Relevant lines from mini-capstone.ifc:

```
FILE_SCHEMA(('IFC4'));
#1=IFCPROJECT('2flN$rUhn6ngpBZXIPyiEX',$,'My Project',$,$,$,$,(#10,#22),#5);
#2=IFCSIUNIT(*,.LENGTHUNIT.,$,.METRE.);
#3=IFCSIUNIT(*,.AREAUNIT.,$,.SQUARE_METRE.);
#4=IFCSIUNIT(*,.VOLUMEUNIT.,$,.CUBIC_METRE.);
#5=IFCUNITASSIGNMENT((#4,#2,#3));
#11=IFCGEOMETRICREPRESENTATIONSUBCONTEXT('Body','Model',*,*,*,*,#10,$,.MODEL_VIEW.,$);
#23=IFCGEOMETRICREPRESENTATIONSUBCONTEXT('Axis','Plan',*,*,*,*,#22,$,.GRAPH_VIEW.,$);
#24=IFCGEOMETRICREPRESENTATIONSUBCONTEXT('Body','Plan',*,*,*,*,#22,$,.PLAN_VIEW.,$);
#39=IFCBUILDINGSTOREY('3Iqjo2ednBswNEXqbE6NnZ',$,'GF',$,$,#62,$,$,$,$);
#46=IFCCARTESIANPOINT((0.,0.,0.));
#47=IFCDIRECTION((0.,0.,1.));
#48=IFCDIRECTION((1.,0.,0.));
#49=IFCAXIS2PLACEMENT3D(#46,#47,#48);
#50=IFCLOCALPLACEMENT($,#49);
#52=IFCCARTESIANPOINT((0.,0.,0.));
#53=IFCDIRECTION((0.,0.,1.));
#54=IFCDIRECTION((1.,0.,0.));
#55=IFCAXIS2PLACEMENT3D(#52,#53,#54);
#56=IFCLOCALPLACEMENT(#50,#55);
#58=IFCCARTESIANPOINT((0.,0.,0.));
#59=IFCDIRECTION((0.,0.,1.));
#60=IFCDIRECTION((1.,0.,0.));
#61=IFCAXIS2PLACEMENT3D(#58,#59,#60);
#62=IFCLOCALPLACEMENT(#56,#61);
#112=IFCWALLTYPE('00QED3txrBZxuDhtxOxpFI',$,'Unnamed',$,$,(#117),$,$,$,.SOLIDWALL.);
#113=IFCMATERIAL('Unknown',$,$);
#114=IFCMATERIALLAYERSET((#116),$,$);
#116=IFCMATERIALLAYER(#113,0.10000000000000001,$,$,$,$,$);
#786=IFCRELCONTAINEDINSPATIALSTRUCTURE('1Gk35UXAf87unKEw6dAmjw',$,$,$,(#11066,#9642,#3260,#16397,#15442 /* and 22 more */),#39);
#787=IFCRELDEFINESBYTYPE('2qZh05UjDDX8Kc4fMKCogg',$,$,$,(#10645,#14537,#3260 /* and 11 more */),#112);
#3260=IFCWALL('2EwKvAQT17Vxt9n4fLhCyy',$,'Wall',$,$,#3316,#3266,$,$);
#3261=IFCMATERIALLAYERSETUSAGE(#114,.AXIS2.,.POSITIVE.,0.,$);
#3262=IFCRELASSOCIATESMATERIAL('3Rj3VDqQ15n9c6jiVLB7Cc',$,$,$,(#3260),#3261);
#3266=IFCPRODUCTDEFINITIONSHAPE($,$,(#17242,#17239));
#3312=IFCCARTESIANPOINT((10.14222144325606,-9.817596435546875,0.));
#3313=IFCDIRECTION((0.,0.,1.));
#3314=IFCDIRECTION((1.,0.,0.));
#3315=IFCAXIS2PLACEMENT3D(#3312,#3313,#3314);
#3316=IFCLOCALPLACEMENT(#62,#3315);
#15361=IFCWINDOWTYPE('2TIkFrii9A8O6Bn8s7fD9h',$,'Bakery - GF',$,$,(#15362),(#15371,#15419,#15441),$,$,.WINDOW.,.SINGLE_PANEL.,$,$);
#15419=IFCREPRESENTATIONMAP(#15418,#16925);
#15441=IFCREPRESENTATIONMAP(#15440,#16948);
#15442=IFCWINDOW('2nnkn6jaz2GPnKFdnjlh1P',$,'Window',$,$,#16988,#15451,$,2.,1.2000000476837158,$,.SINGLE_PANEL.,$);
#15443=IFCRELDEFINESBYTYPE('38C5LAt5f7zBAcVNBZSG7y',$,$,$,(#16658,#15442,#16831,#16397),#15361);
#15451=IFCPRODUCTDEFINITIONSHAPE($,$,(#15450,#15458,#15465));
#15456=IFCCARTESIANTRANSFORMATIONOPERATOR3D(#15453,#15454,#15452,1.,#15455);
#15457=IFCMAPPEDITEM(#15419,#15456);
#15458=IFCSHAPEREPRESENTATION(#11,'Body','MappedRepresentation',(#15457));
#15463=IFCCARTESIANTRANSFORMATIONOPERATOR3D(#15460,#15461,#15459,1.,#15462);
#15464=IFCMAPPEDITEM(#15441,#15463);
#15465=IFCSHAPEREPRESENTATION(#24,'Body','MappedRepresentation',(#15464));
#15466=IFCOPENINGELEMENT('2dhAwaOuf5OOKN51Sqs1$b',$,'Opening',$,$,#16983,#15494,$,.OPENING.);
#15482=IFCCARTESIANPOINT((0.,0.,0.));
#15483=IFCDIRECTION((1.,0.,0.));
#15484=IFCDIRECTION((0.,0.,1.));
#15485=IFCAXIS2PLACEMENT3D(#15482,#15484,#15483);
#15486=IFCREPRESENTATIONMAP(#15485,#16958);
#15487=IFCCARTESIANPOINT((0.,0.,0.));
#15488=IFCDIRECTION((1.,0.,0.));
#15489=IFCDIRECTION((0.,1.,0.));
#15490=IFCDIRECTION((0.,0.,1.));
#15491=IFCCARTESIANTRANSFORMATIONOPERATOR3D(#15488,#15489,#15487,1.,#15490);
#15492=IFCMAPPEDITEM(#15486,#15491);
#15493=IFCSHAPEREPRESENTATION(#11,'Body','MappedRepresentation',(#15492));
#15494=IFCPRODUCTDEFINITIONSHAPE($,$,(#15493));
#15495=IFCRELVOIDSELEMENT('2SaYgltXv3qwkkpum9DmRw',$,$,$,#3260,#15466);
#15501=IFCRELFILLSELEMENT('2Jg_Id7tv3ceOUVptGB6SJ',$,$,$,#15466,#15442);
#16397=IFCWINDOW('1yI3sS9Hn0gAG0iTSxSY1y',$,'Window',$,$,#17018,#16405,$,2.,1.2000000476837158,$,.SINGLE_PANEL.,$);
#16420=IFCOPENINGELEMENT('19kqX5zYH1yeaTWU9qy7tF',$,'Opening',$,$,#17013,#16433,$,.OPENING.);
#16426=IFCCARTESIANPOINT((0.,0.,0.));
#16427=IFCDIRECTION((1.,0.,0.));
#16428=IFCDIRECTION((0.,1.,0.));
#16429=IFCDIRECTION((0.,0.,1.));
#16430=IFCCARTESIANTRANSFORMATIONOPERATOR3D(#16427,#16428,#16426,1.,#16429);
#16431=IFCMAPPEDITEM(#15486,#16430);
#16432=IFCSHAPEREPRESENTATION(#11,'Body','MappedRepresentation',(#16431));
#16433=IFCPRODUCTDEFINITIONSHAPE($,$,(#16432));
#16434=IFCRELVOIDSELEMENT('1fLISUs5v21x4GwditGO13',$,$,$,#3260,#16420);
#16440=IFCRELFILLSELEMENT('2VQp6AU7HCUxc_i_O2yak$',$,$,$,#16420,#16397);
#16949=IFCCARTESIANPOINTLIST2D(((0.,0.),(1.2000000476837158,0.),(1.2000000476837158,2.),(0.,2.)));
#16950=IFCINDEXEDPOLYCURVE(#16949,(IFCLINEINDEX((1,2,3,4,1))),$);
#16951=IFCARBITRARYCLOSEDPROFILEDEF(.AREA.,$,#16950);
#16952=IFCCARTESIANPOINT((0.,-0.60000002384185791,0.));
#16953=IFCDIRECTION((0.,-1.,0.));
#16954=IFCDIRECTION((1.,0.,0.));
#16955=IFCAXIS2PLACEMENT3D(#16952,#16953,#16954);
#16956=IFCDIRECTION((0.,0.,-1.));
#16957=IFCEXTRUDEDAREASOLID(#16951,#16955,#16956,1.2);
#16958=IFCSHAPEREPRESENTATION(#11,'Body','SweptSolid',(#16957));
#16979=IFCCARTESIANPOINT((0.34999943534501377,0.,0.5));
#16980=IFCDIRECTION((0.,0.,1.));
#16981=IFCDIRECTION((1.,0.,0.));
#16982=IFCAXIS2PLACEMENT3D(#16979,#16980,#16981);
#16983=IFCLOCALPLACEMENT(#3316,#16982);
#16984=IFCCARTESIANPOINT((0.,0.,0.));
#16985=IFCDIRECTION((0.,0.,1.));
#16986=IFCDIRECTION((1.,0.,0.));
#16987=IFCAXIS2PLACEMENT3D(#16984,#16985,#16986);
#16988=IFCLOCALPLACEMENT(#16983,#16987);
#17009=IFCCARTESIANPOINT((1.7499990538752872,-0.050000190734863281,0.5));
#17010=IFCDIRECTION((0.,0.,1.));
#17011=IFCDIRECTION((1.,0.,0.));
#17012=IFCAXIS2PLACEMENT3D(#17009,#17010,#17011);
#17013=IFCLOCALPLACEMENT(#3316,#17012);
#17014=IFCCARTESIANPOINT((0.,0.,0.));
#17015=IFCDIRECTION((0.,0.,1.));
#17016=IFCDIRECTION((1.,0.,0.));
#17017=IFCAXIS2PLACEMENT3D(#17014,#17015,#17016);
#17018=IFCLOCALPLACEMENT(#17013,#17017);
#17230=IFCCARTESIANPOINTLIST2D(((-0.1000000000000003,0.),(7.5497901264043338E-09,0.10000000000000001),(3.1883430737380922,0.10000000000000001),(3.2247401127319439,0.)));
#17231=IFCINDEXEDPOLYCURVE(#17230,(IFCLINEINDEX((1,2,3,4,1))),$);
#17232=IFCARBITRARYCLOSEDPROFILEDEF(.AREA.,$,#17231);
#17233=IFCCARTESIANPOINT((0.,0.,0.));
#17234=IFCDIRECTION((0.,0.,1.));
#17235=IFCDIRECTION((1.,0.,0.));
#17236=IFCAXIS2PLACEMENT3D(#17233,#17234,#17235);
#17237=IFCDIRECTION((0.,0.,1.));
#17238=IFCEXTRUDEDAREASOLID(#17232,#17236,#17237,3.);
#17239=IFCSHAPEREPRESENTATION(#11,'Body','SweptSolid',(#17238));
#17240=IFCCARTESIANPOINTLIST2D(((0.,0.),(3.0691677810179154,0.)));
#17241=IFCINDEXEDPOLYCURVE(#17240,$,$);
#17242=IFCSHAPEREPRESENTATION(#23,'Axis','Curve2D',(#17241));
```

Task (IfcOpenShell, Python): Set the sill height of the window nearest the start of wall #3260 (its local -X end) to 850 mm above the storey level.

```python
import numpy as np
import ifcopenshell
import ifcopenshell.api.geometry
import ifcopenshell.geom
import ifcopenshell.util.element
import ifcopenshell.util.placement
import ifcopenshell.util.shape
import ifcopenshell.util.unit

model = ifcopenshell.open("mini-capstone.ifc")
unit_scale = ifcopenshell.util.unit.calculate_unit_scale(model)

window = model.by_guid("2nnkn6jaz2GPnKFdnjlh1P")
opening = window.FillsVoids[0].RelatingOpeningElement
storey = ifcopenshell.util.element.get_container(window, ifc_class="IfcBuildingStorey")
level = ifcopenshell.util.placement.get_local_placement(storey.ObjectPlacement)[2, 3]

# The opening's origin need not be at the sill, so measure its lowest point.
shape = ifcopenshell.geom.create_shape(ifcopenshell.geom.settings(), opening)
bottom = ifcopenshell.util.shape.get_shape_bottom_elevation(shape, shape.geometry) / unit_scale
dz = level + 0.85 / unit_scale - bottom

shift = np.array([0.0, 0.0, dz])
# The window is placed relative to its opening, so it follows when the opening moves.
matrix = ifcopenshell.util.placement.get_local_placement(opening.ObjectPlacement)
matrix[:3, 3] += shift
ifcopenshell.api.geometry.edit_object_placement(
    model, product=opening, matrix=matrix, is_si=False, should_transform_children=True
)

print(f"moved by {dz * unit_scale:+.3f} m")

model.write("mini-capstone-out.ifc")
```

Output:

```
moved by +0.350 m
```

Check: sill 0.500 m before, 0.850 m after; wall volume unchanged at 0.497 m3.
